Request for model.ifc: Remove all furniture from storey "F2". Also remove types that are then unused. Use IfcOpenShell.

First a look at what the model holds.

```python
import ifcopenshell
import ifcopenshell.util.element

model = ifcopenshell.open("model.ifc")
print(model.schema)
storey = next(s for s in model.by_type("IfcBuildingStorey") if s.Name == "F2")
furniture = [e for e in ifcopenshell.util.element.get_decomposition(storey) if e.is_a("IfcFurnishingElement")]
seen = {}
for e in furniture:
    element_type = ifcopenshell.util.element.get_type(e)
    name = element_type.Name if element_type not in (None, e) else None
    seen[name] = seen.get(name, 0) + 1
for name, count in sorted(seen.items(), key=str):
    print(count, "x", name)
```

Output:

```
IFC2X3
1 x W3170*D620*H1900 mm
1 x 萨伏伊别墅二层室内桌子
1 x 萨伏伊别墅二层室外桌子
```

```python
import ifcopenshell
import ifcopenshell.api.root
import ifcopenshell.util.element

model = ifcopenshell.open("model.ifc")

storey = next(s for s in model.by_type("IfcBuildingStorey") if s.Name == "F2")
furniture = [e for e in ifcopenshell.util.element.get_decomposition(storey) if e.is_a("IfcFurnishingElement")]
types = {ifcopenshell.util.element.get_type(e) for e in furniture} - {None, *furniture}

for e in furniture:
    ifcopenshell.api.root.remove_product(model, product=e)
print(len(furniture), "removed")

unused = [t for t in types if not ifcopenshell.util.element.get_types(t)]
for t in unused:
    ifcopenshell.api.root.remove_product(model, product=t)
print(len(unused), "unused types removed")

model.write("model-out.ifc")
```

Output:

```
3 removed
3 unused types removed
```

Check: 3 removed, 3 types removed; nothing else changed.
